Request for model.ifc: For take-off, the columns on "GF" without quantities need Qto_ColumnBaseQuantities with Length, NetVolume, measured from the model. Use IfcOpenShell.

First a look at what the model holds.

```python
import ifcopenshell
import ifcopenshell.util.element
import ifcopenshell.util.unit

model = ifcopenshell.open("model.ifc")
print(model.schema)
for unit_type in ("LENGTHUNIT", "AREAUNIT", "VOLUMEUNIT"):
    print(unit_type, ifcopenshell.util.unit.calculate_unit_scale(model, unit_type))
storey = next(s for s in model.by_type("IfcBuildingStorey") if s.Name == "GF")
columns = [e for e in ifcopenshell.util.element.get_decomposition(storey) if e.is_a("IfcColumn")]
for e in sorted(columns, key=lambda e: e.id()):
    print(e.id(), e.is_a(), e.Name, list(ifcopenshell.util.element.get_psets(e, qtos_only=True)), sep=" | ")
```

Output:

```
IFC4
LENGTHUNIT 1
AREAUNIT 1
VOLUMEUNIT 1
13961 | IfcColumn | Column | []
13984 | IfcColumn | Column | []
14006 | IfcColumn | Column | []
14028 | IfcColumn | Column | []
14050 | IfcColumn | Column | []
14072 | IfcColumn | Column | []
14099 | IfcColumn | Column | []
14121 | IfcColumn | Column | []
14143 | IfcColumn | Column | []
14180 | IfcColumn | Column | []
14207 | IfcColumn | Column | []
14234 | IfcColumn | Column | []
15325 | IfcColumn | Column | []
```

```python
import ifcopenshell
import ifcopenshell.api.pset
import ifcopenshell.geom
import ifcopenshell.util.element
import ifcopenshell.util.shape
import ifcopenshell.util.unit

model = ifcopenshell.open("model.ifc")
unit_scale = ifcopenshell.util.unit.calculate_unit_scale(model)
volume_scale = ifcopenshell.util.unit.calculate_unit_scale(model, "VOLUMEUNIT")
settings = ifcopenshell.geom.settings()

storey = next(s for s in model.by_type("IfcBuildingStorey") if s.Name == "GF")
columns = [e for e in ifcopenshell.util.element.get_decomposition(storey) if e.is_a("IfcColumn")]

for e in sorted(columns, key=lambda e: e.id()):
    if ifcopenshell.util.element.get_psets(e, qtos_only=True, should_inherit=False):
        continue
    # Geometry comes back in metres, in the element's own axes.
    shape = ifcopenshell.geom.create_shape(settings, e)
    values = {
        "Length": ifcopenshell.util.shape.get_z(shape.geometry) / unit_scale,
        "NetVolume": ifcopenshell.util.shape.get_volume(shape.geometry) / volume_scale,
    }
    qto = ifcopenshell.api.pset.add_qto(model, product=e, name="Qto_ColumnBaseQuantities")
    ifcopenshell.api.pset.edit_qto(model, qto=qto, properties=values)
    print(e.id(), {k: round(v, 3) for k, v in values.items()})

model.write("model_rev.ifc")
```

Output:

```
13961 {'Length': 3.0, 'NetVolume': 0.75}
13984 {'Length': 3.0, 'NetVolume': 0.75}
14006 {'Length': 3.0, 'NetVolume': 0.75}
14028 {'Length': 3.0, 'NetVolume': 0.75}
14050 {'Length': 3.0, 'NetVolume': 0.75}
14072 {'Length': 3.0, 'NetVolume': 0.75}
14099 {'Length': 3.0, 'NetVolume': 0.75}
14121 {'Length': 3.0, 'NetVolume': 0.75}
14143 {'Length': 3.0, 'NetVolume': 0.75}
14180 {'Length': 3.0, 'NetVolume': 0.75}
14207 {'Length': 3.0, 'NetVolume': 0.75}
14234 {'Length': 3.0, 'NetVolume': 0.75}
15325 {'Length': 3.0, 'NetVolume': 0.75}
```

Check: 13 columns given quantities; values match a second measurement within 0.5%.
